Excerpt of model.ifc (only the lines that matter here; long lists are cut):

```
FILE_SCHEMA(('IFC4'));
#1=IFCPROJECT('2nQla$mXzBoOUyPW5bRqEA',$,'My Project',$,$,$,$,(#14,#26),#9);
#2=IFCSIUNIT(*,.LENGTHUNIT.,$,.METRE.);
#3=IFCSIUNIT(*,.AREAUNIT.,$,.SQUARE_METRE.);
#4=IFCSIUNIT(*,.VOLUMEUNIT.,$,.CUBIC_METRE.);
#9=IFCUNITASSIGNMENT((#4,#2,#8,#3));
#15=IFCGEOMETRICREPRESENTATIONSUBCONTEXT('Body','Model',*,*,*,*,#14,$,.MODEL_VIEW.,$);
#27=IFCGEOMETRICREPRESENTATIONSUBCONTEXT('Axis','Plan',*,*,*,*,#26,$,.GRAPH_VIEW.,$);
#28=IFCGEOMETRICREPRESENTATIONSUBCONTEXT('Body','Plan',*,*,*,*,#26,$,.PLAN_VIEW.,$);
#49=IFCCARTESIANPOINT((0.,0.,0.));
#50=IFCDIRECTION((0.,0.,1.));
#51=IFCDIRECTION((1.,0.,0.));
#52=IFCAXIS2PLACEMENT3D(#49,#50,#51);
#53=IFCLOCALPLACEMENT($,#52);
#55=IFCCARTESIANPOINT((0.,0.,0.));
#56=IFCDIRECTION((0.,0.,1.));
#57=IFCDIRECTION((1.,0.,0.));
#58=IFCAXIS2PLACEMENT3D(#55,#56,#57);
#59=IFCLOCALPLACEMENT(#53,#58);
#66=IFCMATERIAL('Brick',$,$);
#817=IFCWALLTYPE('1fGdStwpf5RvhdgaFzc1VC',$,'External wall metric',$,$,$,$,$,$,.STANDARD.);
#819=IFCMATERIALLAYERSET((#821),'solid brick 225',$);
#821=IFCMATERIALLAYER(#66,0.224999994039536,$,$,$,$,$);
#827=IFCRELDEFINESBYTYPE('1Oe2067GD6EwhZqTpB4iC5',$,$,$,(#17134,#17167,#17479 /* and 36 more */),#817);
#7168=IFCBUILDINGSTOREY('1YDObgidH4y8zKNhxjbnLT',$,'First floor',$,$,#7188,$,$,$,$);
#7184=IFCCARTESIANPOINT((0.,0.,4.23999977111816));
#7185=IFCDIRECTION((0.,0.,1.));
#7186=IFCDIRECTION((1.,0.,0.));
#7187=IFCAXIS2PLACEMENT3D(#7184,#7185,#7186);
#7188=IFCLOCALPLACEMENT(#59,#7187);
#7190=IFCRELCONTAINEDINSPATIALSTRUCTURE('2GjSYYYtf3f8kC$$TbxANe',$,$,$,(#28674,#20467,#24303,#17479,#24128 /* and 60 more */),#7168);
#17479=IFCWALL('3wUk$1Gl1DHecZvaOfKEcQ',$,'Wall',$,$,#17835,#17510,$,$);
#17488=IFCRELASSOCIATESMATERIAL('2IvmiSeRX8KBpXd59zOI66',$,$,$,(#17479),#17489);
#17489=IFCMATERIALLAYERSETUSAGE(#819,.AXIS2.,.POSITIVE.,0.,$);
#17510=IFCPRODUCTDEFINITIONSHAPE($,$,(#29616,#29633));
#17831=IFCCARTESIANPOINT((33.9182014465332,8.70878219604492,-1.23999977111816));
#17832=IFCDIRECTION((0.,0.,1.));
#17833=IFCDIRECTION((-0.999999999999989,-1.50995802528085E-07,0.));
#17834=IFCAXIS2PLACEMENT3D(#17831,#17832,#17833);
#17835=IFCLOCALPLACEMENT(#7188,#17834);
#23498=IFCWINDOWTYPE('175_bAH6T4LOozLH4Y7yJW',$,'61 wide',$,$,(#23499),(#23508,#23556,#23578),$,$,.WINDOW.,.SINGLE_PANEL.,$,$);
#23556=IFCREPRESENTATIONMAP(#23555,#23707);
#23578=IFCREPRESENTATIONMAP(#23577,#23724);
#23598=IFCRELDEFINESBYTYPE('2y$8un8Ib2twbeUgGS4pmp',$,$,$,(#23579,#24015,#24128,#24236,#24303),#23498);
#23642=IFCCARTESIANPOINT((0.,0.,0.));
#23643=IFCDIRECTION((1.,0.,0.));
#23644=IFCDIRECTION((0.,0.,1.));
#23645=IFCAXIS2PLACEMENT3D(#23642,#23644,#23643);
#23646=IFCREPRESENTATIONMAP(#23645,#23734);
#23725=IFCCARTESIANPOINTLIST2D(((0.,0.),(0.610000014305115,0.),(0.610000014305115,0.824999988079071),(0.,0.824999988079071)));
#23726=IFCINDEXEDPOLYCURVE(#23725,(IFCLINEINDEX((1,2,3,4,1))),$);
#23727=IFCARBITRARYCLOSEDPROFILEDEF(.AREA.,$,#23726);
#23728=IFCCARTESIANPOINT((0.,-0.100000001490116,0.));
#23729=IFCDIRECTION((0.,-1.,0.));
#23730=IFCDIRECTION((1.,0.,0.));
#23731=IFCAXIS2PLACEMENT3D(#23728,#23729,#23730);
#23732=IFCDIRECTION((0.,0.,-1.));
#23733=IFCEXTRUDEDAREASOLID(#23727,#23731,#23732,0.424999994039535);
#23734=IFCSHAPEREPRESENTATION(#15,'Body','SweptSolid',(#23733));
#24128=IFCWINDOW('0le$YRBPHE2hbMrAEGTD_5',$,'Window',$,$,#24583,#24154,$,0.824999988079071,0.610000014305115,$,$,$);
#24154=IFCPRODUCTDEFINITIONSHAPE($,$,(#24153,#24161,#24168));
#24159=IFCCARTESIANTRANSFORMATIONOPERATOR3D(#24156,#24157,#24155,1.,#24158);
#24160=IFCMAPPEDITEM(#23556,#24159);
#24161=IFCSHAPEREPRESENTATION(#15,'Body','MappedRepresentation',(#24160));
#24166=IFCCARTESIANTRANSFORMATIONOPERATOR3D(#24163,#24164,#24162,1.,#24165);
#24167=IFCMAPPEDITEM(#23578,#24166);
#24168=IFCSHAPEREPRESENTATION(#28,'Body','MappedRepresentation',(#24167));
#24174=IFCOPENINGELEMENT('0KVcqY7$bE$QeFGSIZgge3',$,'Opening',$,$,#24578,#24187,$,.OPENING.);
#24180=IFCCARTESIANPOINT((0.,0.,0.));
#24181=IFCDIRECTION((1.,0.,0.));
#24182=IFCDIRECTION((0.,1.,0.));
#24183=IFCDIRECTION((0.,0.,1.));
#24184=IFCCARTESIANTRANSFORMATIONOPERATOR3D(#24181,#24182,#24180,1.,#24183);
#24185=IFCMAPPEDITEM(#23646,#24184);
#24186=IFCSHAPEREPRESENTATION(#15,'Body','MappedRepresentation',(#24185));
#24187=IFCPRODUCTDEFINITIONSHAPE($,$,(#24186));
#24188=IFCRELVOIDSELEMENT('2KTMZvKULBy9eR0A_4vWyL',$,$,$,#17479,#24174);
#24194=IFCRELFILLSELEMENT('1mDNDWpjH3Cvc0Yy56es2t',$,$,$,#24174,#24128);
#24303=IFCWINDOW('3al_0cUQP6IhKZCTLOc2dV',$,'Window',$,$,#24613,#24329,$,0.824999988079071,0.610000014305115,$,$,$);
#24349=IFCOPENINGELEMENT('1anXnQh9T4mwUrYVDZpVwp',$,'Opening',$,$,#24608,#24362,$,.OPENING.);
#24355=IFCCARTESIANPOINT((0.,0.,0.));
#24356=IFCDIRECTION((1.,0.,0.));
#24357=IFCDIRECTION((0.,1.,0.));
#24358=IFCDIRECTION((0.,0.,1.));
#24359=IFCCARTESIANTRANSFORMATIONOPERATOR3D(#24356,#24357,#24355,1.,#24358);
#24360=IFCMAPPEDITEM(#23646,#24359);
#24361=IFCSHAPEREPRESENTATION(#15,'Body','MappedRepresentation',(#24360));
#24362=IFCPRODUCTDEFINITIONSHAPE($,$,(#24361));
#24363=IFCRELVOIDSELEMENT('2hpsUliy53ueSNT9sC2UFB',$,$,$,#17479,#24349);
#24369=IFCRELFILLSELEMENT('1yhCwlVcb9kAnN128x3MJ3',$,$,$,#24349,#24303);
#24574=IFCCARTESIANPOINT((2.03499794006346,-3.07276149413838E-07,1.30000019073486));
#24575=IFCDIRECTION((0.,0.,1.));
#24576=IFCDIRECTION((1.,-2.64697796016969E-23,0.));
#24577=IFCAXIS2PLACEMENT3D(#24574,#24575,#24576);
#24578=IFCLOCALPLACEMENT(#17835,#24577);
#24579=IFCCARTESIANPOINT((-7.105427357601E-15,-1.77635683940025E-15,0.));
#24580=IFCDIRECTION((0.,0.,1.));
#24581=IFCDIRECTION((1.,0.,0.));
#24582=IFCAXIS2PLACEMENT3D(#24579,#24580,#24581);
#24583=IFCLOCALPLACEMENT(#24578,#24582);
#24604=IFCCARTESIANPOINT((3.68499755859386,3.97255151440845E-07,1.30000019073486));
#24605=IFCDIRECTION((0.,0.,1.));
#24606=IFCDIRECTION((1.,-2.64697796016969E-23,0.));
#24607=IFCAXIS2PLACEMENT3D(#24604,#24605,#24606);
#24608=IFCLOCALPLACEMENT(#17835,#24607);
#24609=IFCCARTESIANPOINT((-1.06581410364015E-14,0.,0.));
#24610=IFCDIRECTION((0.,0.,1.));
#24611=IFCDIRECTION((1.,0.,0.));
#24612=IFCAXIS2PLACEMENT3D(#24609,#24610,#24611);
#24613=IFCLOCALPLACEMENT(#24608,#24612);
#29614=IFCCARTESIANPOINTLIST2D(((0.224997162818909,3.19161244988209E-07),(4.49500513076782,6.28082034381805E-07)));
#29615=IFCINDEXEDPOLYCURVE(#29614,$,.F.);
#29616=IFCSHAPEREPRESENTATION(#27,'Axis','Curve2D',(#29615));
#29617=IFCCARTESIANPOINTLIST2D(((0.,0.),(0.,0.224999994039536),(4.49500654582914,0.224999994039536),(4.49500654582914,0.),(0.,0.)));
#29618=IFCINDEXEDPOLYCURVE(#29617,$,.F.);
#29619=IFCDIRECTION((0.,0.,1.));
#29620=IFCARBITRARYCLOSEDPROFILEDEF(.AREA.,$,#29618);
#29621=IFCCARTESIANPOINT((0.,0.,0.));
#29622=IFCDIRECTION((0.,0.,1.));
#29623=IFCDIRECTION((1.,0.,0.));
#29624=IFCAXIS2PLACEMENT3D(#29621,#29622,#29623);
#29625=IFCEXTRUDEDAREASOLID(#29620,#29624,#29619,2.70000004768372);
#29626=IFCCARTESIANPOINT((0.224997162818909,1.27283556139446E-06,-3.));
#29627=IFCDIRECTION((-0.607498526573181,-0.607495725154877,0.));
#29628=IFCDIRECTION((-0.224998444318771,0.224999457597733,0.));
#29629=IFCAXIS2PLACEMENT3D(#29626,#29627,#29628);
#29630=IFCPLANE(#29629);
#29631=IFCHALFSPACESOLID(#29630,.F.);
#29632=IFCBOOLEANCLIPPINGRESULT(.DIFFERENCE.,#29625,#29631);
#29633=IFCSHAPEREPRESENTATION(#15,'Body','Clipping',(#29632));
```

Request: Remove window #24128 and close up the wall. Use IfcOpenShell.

```python
import ifcopenshell
import ifcopenshell.api.feature
import ifcopenshell.api.root
import ifcopenshell.geom
import ifcopenshell.util.shape

model = ifcopenshell.open("model.ifc")
settings = ifcopenshell.geom.settings()


def volume(element):
    """Net volume in cubic metres, openings subtracted."""
    shape = ifcopenshell.geom.create_shape(settings, element)
    return ifcopenshell.util.shape.get_volume(shape.geometry)


window = model.by_guid("0le$YRBPHE2hbMrAEGTD_5")
opening = window.FillsVoids[0].RelatingOpeningElement
wall = opening.VoidsElements[0].RelatingBuildingElement
before = volume(wall)

ifcopenshell.api.root.remove_product(model, product=window)
ifcopenshell.api.feature.remove_feature(model, feature=opening)

after = volume(wall)

print(f"wall volume {before:.3f} -> {after:.3f} m3")

model.write("model_updated.ifc")
```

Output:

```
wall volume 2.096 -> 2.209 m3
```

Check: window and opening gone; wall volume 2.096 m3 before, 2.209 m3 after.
